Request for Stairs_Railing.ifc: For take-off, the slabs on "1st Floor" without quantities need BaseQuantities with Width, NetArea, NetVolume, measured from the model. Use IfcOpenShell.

First a look at what the model holds.

```python
import ifcopenshell
import ifcopenshell.util.element
import ifcopenshell.util.unit

model = ifcopenshell.open("Stairs_Railing.ifc")
print(model.schema)
for unit_type in ("LENGTHUNIT", "AREAUNIT", "VOLUMEUNIT"):
    print(unit_type, ifcopenshell.util.unit.calculate_unit_scale(model, unit_type))
storey = next(s for s in model.by_type("IfcBuildingStorey") if s.Name == "1st Floor")
slabs = [e for e in ifcopenshell.util.element.get_decomposition(storey) if e.is_a("IfcSlab")]
for e in sorted(slabs, key=lambda e: e.id()):
    print(e.id(), e.is_a(), e.Name, list(ifcopenshell.util.element.get_psets(e, qtos_only=True)), sep=" | ")
```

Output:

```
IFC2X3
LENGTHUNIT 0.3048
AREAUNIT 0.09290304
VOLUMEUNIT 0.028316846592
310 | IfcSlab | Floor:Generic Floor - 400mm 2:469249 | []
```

```python
import ifcopenshell
import ifcopenshell.api.pset
import ifcopenshell.geom
import ifcopenshell.util.element
import ifcopenshell.util.shape
import ifcopenshell.util.unit

model = ifcopenshell.open("Stairs_Railing.ifc")
unit_scale = ifcopenshell.util.unit.calculate_unit_scale(model)
area_scale = ifcopenshell.util.unit.calculate_unit_scale(model, "AREAUNIT")
volume_scale = ifcopenshell.util.unit.calculate_unit_scale(model, "VOLUMEUNIT")
settings = ifcopenshell.geom.settings()

storey = next(s for s in model.by_type("IfcBuildingStorey") if s.Name == "1st Floor")
slabs = [e for e in ifcopenshell.util.element.get_decomposition(storey) if e.is_a("IfcSlab")]

for e in sorted(slabs, key=lambda e: e.id()):
    if ifcopenshell.util.element.get_psets(e, qtos_only=True, should_inherit=False):
        continue
    # Geometry comes back in metres, in the element's own axes.
    shape = ifcopenshell.geom.create_shape(settings, e)
    values = {
        "Width": ifcopenshell.util.shape.get_z(shape.geometry) / unit_scale,
        "NetArea": ifcopenshell.util.shape.get_footprint_area(shape.geometry) / area_scale,
        "NetVolume": ifcopenshell.util.shape.get_volume(shape.geometry) / volume_scale,
    }
    qto = ifcopenshell.api.pset.add_qto(model, product=e, name="BaseQuantities")
    ifcopenshell.api.pset.edit_qto(model, qto=qto, properties=values)
    print(e.id(), {k: round(v, 3) for k, v in values.items()})

model.write("Stairs_Railing_v2.ifc")
```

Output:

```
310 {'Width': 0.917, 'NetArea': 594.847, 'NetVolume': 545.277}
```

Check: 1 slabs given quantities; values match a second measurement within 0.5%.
